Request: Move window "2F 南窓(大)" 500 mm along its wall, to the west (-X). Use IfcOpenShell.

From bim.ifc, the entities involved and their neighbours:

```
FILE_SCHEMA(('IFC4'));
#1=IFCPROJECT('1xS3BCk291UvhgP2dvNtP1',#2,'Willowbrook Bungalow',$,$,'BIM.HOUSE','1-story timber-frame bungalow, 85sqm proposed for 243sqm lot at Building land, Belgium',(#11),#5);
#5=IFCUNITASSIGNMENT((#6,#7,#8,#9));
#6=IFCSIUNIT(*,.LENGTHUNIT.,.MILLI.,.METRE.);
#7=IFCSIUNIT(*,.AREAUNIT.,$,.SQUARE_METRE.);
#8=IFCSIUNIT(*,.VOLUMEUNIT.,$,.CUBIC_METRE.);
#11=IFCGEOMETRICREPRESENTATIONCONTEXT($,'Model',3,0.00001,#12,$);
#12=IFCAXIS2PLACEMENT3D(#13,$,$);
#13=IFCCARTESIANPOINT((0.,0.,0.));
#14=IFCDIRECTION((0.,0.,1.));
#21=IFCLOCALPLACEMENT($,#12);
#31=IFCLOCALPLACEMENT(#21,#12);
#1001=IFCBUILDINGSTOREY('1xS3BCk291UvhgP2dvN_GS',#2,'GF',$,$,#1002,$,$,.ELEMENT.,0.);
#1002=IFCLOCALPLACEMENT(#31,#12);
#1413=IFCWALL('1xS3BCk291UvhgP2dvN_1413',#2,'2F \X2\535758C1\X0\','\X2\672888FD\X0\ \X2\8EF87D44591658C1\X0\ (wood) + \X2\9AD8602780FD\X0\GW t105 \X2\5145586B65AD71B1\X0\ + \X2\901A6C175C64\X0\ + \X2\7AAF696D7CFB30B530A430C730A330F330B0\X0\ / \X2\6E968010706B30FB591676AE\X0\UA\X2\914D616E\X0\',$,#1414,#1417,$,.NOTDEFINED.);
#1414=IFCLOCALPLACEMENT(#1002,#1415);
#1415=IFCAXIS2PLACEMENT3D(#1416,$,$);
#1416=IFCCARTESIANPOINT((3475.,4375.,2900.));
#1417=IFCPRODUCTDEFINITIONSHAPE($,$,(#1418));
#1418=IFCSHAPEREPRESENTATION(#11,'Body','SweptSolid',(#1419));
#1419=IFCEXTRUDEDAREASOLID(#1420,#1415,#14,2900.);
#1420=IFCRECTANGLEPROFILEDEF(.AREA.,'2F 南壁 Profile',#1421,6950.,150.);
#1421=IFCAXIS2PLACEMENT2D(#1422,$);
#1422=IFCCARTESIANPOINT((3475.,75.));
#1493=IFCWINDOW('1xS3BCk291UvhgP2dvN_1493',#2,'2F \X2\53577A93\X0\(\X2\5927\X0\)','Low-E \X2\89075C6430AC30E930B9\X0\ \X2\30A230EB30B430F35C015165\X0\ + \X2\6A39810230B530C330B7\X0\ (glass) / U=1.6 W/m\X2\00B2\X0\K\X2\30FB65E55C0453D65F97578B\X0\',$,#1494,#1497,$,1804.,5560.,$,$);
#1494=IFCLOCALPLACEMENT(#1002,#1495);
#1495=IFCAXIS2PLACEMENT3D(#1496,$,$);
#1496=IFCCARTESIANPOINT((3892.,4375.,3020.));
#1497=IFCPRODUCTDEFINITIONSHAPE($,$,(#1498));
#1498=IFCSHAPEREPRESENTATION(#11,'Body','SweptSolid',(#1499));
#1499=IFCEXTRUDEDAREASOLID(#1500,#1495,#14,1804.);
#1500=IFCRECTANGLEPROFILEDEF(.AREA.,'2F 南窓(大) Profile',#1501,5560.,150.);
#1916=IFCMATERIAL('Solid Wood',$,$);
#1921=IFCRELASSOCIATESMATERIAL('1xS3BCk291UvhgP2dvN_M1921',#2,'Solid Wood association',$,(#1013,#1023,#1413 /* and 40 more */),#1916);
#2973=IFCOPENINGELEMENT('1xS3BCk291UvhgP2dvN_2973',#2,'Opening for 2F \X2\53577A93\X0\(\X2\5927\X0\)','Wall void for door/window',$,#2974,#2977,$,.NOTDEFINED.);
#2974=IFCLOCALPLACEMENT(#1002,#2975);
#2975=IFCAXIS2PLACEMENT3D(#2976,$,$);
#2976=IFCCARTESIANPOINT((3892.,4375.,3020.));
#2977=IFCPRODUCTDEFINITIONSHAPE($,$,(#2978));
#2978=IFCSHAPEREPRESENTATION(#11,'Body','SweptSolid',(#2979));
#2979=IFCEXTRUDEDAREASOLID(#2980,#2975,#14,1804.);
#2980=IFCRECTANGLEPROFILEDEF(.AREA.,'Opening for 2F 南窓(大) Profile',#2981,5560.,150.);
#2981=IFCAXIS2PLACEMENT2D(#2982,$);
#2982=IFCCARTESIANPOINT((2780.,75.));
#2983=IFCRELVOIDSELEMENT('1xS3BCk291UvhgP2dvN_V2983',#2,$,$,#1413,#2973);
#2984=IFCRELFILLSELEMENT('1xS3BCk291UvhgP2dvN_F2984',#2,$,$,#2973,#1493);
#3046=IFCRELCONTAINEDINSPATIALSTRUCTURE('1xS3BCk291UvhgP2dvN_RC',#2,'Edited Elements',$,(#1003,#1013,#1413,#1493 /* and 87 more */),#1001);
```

```python
import ifcopenshell
import ifcopenshell.api.geometry
import ifcopenshell.util.placement
import ifcopenshell.util.unit

model = ifcopenshell.open("bim.ifc")
unit_scale = ifcopenshell.util.unit.calculate_unit_scale(model)

window = model.by_guid("1xS3BCk291UvhgP2dvN_1493")
opening = window.FillsVoids[0].RelatingOpeningElement
wall = opening.VoidsElements[0].RelatingBuildingElement

wall_matrix = ifcopenshell.util.placement.get_local_placement(wall.ObjectPlacement)
shift = wall_matrix[:3, 0] * -0.5 / unit_scale
before = ifcopenshell.util.placement.get_local_placement(window.ObjectPlacement)[:3, 3].copy()

# The window is not placed relative to its opening, so move both.
for product in (opening, window):
    matrix = ifcopenshell.util.placement.get_local_placement(product.ObjectPlacement)
    matrix[:3, 3] += shift
    ifcopenshell.api.geometry.edit_object_placement(model, product=product, matrix=matrix, is_si=False)

after = ifcopenshell.util.placement.get_local_placement(window.ObjectPlacement)[:3, 3]
print("window moved by", (after - before).round(3) + 0.0)

model.write("bim_edited.ifc")
```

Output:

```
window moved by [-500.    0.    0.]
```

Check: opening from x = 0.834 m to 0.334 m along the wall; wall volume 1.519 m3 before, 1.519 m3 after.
